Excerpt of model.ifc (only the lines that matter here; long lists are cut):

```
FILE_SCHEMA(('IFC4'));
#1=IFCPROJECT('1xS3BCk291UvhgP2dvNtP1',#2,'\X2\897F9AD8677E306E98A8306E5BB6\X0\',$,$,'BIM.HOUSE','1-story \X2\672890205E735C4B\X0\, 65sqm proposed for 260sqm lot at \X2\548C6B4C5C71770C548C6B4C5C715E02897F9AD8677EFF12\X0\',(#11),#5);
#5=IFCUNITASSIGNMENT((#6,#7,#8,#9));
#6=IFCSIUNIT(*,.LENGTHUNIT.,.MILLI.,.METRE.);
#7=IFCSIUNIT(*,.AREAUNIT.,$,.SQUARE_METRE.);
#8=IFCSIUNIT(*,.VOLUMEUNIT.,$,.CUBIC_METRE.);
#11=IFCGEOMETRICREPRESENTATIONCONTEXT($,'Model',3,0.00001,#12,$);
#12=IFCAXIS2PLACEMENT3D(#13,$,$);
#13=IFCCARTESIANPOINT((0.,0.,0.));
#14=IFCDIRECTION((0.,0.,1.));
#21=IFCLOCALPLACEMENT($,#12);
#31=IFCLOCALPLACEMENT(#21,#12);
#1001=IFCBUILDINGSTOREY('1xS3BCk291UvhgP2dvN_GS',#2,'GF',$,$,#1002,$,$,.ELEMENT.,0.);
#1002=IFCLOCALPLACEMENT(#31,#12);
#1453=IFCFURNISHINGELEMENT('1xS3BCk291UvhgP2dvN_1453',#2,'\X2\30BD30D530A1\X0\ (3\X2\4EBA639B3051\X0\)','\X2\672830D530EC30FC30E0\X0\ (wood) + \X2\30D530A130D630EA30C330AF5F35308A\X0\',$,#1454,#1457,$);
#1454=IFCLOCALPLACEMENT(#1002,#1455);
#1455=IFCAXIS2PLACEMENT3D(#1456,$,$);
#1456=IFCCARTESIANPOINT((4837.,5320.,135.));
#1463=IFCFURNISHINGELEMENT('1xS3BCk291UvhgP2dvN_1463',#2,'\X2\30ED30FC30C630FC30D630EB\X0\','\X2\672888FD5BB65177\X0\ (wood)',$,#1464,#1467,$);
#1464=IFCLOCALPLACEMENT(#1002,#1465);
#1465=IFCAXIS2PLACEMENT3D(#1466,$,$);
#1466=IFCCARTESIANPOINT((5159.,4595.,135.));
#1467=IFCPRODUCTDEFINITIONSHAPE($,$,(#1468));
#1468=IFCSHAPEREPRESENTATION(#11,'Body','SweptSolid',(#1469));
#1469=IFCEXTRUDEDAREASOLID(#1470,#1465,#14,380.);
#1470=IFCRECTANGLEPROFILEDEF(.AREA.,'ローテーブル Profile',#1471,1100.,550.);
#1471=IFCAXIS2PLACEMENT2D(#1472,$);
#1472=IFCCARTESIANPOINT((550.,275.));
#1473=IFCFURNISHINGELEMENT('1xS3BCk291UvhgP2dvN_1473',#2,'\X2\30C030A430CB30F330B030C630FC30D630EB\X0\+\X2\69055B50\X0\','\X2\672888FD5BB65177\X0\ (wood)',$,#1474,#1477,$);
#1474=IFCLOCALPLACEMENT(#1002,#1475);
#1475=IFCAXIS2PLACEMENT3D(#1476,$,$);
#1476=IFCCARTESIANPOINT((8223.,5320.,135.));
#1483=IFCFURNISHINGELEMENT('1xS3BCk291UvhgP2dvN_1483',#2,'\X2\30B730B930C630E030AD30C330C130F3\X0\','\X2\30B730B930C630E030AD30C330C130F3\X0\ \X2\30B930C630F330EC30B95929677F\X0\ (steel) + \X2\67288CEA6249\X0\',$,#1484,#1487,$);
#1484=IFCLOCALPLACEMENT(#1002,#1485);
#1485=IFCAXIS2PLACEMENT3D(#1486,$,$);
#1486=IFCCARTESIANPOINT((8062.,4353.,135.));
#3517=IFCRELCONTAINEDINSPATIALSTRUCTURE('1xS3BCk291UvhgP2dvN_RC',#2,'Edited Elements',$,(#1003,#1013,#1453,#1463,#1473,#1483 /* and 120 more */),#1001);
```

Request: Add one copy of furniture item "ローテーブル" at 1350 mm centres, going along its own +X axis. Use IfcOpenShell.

```python
import ifcopenshell
import ifcopenshell.api.geometry
import ifcopenshell.api.root
import ifcopenshell.util.element
import ifcopenshell.util.placement
import ifcopenshell.util.unit

model = ifcopenshell.open("model.ifc")
unit_scale = ifcopenshell.util.unit.calculate_unit_scale(model)


def reuse_history(source, copy):
    """copy_class also copies each property set's owner history, people and application; keep the originals."""
    for rel in copy.IsDefinedBy:
        if rel.is_a("IfcRelDefinesByProperties") and (history := rel.RelatingPropertyDefinition.OwnerHistory):
            rel.RelatingPropertyDefinition.OwnerHistory = source.OwnerHistory
            ifcopenshell.util.element.remove_deep2(model, history)


source = model.by_guid("1xS3BCk291UvhgP2dvN_1463")
base = ifcopenshell.util.placement.get_local_placement(source.ObjectPlacement)
step = base[:3, 0] * 1.35 / unit_scale

for i in range(1, 2):
    copy = ifcopenshell.api.root.copy_class(model, product=source)
    copy.Representation = ifcopenshell.util.element.copy_deep(
        model, source.Representation, exclude=["IfcGeometricRepresentationContext", "IfcRepresentationMap"]
    )
    reuse_history(source, copy)
    matrix = base.copy()
    matrix[:3, 3] += i * step
    print("added at", matrix[:3, 3].round(3) + 0.0)
    ifcopenshell.api.geometry.edit_object_placement(model, product=copy, matrix=matrix, is_si=False)

model.write("model-out.ifc")
```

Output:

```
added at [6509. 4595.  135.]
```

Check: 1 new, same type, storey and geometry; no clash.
